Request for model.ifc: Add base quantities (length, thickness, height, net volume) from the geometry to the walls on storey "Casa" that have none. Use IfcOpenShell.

First a look at what the model holds.

```python
import ifcopenshell
import ifcopenshell.util.element
import ifcopenshell.util.unit

model = ifcopenshell.open("model.ifc")
print(model.schema)
for unit_type in ("LENGTHUNIT", "AREAUNIT", "VOLUMEUNIT"):
    print(unit_type, ifcopenshell.util.unit.calculate_unit_scale(model, unit_type))
storey = next(s for s in model.by_type("IfcBuildingStorey") if s.Name == "Casa")
walls = [e for e in ifcopenshell.util.element.get_decomposition(storey) if e.is_a("IfcWall")]
for e in sorted(walls, key=lambda e: e.id()):
    print(e.id(), e.is_a(), e.Name, list(ifcopenshell.util.element.get_psets(e, qtos_only=True)), sep=" | ")
```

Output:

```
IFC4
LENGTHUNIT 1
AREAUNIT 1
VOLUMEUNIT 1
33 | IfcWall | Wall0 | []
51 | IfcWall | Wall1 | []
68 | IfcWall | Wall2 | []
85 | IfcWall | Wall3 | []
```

```python
import ifcopenshell
import ifcopenshell.api.pset
import ifcopenshell.geom
import ifcopenshell.util.element
import ifcopenshell.util.shape
import ifcopenshell.util.unit

model = ifcopenshell.open("model.ifc")
unit_scale = ifcopenshell.util.unit.calculate_unit_scale(model)
volume_scale = ifcopenshell.util.unit.calculate_unit_scale(model, "VOLUMEUNIT")
settings = ifcopenshell.geom.settings()

storey = next(s for s in model.by_type("IfcBuildingStorey") if s.Name == "Casa")
walls = [e for e in ifcopenshell.util.element.get_decomposition(storey) if e.is_a("IfcWall")]

for e in sorted(walls, key=lambda e: e.id()):
    if ifcopenshell.util.element.get_psets(e, qtos_only=True, should_inherit=False):
        continue
    # Geometry comes back in metres, in the element's own axes.
    shape = ifcopenshell.geom.create_shape(settings, e)
    values = {
        "Length": ifcopenshell.util.shape.get_x(shape.geometry) / unit_scale,
        "Width": ifcopenshell.util.shape.get_y(shape.geometry) / unit_scale,
        "Height": ifcopenshell.util.shape.get_z(shape.geometry) / unit_scale,
        "NetVolume": ifcopenshell.util.shape.get_volume(shape.geometry) / volume_scale,
    }
    qto = ifcopenshell.api.pset.add_qto(model, product=e, name="Qto_WallBaseQuantities")
    ifcopenshell.api.pset.edit_qto(model, qto=qto, properties=values)
    print(e.id(), {k: round(v, 3) for k, v in values.items()})

model.write("model_updated.ifc")
```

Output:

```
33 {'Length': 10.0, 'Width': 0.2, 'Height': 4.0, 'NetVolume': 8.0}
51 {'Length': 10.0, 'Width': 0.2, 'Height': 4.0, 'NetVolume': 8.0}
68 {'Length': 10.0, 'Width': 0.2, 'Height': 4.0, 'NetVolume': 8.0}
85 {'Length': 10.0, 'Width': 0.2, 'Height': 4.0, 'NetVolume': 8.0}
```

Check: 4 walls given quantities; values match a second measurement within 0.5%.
